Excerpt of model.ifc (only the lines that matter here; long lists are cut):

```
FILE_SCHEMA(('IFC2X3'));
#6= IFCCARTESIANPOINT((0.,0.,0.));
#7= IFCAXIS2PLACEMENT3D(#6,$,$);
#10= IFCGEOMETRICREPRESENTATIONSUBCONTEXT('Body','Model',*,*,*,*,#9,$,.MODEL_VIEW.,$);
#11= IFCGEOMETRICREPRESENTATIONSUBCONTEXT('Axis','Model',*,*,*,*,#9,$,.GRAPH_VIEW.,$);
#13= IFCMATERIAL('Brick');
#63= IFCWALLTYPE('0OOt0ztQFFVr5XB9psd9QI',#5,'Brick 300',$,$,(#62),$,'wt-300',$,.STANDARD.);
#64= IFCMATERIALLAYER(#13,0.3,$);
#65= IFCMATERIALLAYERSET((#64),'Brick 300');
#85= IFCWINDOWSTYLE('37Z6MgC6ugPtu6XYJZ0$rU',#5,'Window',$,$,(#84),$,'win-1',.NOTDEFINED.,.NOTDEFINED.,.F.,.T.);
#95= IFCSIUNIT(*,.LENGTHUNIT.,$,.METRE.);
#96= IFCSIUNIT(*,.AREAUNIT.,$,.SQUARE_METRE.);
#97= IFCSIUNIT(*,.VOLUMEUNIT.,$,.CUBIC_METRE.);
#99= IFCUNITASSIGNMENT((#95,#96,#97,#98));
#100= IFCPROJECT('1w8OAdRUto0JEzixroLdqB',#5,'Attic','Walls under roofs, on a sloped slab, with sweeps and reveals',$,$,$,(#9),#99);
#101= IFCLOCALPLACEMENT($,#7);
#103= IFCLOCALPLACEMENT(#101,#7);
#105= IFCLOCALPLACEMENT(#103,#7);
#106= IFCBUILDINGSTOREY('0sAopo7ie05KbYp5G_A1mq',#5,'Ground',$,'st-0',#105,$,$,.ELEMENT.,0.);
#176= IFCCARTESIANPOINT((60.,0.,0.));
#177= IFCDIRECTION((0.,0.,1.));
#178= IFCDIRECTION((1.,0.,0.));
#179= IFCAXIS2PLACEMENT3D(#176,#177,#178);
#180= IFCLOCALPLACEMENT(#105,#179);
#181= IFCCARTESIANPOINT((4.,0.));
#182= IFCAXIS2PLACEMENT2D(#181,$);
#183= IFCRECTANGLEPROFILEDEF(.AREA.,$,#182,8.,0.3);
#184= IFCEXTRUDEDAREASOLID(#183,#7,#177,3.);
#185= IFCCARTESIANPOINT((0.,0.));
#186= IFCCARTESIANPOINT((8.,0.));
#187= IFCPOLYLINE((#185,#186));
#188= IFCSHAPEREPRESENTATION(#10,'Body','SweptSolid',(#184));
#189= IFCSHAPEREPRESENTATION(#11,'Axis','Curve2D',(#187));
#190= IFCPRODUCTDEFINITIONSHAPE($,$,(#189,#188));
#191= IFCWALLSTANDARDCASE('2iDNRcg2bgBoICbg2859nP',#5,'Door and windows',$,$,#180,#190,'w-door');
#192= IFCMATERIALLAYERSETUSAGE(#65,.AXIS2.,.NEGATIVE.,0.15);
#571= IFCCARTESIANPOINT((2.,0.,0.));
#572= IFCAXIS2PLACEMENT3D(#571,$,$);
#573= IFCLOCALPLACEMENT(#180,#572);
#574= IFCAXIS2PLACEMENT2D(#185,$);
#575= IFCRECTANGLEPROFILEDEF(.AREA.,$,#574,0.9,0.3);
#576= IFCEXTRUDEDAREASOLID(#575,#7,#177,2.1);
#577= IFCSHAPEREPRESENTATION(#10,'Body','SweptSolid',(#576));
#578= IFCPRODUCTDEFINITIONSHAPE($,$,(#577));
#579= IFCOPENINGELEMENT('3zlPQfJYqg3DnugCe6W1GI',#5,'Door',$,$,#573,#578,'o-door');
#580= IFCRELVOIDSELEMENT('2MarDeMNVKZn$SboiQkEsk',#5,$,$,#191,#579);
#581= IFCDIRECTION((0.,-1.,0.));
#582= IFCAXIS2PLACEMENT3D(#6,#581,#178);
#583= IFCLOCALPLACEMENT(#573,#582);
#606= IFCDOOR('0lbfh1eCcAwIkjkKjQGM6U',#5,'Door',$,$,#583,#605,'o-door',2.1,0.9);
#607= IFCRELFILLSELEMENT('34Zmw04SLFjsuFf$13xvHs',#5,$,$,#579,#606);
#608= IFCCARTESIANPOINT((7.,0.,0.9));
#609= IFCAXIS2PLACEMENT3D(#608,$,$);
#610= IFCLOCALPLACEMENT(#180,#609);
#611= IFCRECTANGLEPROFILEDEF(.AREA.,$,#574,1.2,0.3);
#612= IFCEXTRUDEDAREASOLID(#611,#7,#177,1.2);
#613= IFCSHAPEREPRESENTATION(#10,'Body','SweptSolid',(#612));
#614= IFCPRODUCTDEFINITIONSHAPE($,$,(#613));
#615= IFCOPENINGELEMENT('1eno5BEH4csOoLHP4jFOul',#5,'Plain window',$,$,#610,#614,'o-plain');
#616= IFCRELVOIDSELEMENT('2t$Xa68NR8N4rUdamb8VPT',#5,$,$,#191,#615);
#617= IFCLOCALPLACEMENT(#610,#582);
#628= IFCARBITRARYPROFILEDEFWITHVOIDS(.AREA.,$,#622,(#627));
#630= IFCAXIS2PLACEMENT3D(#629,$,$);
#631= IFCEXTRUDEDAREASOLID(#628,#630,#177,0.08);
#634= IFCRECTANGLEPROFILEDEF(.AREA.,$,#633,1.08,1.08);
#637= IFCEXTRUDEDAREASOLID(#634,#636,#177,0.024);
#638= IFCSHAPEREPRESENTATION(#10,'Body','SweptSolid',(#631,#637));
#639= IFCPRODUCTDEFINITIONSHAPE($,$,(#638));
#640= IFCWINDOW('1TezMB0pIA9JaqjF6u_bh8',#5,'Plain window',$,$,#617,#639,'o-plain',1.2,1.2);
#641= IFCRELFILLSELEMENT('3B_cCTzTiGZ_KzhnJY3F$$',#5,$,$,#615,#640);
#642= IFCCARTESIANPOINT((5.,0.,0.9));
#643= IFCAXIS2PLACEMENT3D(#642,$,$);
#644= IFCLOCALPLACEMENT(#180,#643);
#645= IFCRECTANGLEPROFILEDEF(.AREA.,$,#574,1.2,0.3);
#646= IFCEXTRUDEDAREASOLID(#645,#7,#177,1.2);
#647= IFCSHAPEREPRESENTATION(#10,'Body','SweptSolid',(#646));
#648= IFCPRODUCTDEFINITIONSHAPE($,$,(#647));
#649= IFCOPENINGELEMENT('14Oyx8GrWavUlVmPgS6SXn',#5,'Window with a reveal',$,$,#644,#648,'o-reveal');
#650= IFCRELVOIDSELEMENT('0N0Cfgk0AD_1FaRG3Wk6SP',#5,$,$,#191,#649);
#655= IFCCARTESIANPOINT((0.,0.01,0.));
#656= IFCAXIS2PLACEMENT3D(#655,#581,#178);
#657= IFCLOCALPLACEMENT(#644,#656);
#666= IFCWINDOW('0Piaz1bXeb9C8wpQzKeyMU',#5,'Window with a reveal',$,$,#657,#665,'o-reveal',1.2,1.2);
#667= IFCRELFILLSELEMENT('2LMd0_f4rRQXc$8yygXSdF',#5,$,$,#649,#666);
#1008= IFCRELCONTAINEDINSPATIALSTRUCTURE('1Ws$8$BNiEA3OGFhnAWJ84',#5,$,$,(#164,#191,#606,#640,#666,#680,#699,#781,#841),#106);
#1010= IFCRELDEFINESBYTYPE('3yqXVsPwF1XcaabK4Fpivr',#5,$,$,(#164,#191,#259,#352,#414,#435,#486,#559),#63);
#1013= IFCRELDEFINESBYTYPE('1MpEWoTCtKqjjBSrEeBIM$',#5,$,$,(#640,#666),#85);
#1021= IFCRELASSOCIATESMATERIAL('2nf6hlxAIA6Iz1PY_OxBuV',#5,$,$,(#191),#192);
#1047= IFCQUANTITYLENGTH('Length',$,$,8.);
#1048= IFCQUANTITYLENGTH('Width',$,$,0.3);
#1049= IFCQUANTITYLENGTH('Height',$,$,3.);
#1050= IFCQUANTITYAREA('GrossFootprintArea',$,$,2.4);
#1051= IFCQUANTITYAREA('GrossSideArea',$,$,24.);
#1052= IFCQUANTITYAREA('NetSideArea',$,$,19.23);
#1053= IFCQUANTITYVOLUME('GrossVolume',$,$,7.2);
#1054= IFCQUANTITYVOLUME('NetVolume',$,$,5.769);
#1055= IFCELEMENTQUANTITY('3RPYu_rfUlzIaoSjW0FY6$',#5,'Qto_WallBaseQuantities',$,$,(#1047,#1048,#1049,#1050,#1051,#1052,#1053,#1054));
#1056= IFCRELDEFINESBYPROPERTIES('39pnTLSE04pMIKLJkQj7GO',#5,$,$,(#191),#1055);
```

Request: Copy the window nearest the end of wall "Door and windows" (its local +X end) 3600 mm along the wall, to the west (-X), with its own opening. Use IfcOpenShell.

```python
import ifcopenshell
import ifcopenshell.api.feature
import ifcopenshell.api.geometry
import ifcopenshell.api.pset
import ifcopenshell.api.root
import ifcopenshell.geom
import ifcopenshell.util.element
import ifcopenshell.util.placement
import ifcopenshell.util.shape
import ifcopenshell.util.unit

model = ifcopenshell.open("model.ifc")
unit_scale = ifcopenshell.util.unit.calculate_unit_scale(model)
area_scale = ifcopenshell.util.unit.calculate_unit_scale(model, "AREAUNIT")
volume_scale = ifcopenshell.util.unit.calculate_unit_scale(model, "VOLUMEUNIT")
settings = ifcopenshell.geom.settings()


def volume(element):
    """Net volume in cubic metres, openings subtracted."""
    shape = ifcopenshell.geom.create_shape(settings, element)
    return ifcopenshell.util.shape.get_volume(shape.geometry)


def reuse_history(source, copy):
    """copy_class also copies each property set's owner history, people and application; keep the originals."""
    for rel in copy.IsDefinedBy:
        if rel.is_a("IfcRelDefinesByProperties") and (history := rel.RelatingPropertyDefinition.OwnerHistory):
            rel.RelatingPropertyDefinition.OwnerHistory = source.OwnerHistory
            ifcopenshell.util.element.remove_deep2(model, history)


window = model.by_guid("1TezMB0pIA9JaqjF6u_bh8")
opening = window.FillsVoids[0].RelatingOpeningElement
wall = opening.VoidsElements[0].RelatingBuildingElement
before = volume(wall)
shift = ifcopenshell.util.placement.get_local_placement(wall.ObjectPlacement)[:3, 0] * -3.6 / unit_scale

# copy_class copies the void relationship, type, container and properties, but no geometry.
new_opening = ifcopenshell.api.root.copy_class(model, product=opening)
new_opening.Representation = ifcopenshell.util.element.copy_deep(
    model, opening.Representation, exclude=["IfcGeometricRepresentationContext", "IfcRepresentationMap"]
)
new_opening.Tag = None
new_window = ifcopenshell.api.root.copy_class(model, product=window)
new_window.Representation = ifcopenshell.util.element.copy_deep(
    model, window.Representation, exclude=["IfcGeometricRepresentationContext", "IfcRepresentationMap"]
)
new_window.Tag = None
reuse_history(window, new_window)
fills = ifcopenshell.api.feature.add_filling(model, opening=new_opening, element=new_window)
fills.OwnerHistory = new_window.OwnerHistory  # required in IFC2X3

for old, new in ((opening, new_opening), (window, new_window)):
    matrix = ifcopenshell.util.placement.get_local_placement(old.ObjectPlacement)
    matrix[:3, 3] += shift
    ifcopenshell.api.geometry.edit_object_placement(model, product=new, matrix=matrix, is_si=False)

after = volume(wall)
thickness = 0.3  # wall thickness in metres

# Update the wall's stored quantities.
qto = model.by_id(ifcopenshell.util.element.get_pset(wall, "Qto_WallBaseQuantities", should_inherit=False)["id"])
ifcopenshell.api.pset.edit_qto(model, qto=qto, properties={
    "NetSideArea": after / thickness / area_scale,
    "NetVolume": after / volume_scale,
})

print(f"wall volume {before:.3f} -> {after:.3f} m3")

model.write("model_v2.ifc")
```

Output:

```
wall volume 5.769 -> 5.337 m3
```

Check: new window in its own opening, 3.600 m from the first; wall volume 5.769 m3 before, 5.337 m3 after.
